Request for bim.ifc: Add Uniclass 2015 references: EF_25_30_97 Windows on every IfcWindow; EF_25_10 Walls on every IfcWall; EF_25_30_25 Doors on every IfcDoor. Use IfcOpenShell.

First a look at what the model holds.

```python
import ifcopenshell

model = ifcopenshell.open("bim.ifc")
print(model.schema)
print("classifications:", [c.Name for c in model.by_type("IfcClassification")])
for ifc_class in ("IfcDoor", "IfcRoof", "IfcStair", "IfcWall", "IfcWindow"):
    print(ifc_class, len(model.by_type(ifc_class)))
```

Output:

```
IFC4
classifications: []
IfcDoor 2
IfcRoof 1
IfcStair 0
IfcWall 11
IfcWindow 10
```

```python
import ifcopenshell
import ifcopenshell.api.classification

model = ifcopenshell.open("bim.ifc")

system = ifcopenshell.api.classification.add_classification(model, classification="Uniclass 2015")

codes = {
    "IfcWindow": ("EF_25_30_97", "Windows"),
    "IfcWall": ("EF_25_10", "Walls"),
    "IfcDoor": ("EF_25_30_25", "Doors"),
}
for ifc_class, (code, name) in codes.items():
    products = model.by_type(ifc_class)
    ifcopenshell.api.classification.add_reference(
        model, products=products, classification=system, identification=code, name=name
    )
    print(code, len(products))

model.write("bim-out.ifc")
```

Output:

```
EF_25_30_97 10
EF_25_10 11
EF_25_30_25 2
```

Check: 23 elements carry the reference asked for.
